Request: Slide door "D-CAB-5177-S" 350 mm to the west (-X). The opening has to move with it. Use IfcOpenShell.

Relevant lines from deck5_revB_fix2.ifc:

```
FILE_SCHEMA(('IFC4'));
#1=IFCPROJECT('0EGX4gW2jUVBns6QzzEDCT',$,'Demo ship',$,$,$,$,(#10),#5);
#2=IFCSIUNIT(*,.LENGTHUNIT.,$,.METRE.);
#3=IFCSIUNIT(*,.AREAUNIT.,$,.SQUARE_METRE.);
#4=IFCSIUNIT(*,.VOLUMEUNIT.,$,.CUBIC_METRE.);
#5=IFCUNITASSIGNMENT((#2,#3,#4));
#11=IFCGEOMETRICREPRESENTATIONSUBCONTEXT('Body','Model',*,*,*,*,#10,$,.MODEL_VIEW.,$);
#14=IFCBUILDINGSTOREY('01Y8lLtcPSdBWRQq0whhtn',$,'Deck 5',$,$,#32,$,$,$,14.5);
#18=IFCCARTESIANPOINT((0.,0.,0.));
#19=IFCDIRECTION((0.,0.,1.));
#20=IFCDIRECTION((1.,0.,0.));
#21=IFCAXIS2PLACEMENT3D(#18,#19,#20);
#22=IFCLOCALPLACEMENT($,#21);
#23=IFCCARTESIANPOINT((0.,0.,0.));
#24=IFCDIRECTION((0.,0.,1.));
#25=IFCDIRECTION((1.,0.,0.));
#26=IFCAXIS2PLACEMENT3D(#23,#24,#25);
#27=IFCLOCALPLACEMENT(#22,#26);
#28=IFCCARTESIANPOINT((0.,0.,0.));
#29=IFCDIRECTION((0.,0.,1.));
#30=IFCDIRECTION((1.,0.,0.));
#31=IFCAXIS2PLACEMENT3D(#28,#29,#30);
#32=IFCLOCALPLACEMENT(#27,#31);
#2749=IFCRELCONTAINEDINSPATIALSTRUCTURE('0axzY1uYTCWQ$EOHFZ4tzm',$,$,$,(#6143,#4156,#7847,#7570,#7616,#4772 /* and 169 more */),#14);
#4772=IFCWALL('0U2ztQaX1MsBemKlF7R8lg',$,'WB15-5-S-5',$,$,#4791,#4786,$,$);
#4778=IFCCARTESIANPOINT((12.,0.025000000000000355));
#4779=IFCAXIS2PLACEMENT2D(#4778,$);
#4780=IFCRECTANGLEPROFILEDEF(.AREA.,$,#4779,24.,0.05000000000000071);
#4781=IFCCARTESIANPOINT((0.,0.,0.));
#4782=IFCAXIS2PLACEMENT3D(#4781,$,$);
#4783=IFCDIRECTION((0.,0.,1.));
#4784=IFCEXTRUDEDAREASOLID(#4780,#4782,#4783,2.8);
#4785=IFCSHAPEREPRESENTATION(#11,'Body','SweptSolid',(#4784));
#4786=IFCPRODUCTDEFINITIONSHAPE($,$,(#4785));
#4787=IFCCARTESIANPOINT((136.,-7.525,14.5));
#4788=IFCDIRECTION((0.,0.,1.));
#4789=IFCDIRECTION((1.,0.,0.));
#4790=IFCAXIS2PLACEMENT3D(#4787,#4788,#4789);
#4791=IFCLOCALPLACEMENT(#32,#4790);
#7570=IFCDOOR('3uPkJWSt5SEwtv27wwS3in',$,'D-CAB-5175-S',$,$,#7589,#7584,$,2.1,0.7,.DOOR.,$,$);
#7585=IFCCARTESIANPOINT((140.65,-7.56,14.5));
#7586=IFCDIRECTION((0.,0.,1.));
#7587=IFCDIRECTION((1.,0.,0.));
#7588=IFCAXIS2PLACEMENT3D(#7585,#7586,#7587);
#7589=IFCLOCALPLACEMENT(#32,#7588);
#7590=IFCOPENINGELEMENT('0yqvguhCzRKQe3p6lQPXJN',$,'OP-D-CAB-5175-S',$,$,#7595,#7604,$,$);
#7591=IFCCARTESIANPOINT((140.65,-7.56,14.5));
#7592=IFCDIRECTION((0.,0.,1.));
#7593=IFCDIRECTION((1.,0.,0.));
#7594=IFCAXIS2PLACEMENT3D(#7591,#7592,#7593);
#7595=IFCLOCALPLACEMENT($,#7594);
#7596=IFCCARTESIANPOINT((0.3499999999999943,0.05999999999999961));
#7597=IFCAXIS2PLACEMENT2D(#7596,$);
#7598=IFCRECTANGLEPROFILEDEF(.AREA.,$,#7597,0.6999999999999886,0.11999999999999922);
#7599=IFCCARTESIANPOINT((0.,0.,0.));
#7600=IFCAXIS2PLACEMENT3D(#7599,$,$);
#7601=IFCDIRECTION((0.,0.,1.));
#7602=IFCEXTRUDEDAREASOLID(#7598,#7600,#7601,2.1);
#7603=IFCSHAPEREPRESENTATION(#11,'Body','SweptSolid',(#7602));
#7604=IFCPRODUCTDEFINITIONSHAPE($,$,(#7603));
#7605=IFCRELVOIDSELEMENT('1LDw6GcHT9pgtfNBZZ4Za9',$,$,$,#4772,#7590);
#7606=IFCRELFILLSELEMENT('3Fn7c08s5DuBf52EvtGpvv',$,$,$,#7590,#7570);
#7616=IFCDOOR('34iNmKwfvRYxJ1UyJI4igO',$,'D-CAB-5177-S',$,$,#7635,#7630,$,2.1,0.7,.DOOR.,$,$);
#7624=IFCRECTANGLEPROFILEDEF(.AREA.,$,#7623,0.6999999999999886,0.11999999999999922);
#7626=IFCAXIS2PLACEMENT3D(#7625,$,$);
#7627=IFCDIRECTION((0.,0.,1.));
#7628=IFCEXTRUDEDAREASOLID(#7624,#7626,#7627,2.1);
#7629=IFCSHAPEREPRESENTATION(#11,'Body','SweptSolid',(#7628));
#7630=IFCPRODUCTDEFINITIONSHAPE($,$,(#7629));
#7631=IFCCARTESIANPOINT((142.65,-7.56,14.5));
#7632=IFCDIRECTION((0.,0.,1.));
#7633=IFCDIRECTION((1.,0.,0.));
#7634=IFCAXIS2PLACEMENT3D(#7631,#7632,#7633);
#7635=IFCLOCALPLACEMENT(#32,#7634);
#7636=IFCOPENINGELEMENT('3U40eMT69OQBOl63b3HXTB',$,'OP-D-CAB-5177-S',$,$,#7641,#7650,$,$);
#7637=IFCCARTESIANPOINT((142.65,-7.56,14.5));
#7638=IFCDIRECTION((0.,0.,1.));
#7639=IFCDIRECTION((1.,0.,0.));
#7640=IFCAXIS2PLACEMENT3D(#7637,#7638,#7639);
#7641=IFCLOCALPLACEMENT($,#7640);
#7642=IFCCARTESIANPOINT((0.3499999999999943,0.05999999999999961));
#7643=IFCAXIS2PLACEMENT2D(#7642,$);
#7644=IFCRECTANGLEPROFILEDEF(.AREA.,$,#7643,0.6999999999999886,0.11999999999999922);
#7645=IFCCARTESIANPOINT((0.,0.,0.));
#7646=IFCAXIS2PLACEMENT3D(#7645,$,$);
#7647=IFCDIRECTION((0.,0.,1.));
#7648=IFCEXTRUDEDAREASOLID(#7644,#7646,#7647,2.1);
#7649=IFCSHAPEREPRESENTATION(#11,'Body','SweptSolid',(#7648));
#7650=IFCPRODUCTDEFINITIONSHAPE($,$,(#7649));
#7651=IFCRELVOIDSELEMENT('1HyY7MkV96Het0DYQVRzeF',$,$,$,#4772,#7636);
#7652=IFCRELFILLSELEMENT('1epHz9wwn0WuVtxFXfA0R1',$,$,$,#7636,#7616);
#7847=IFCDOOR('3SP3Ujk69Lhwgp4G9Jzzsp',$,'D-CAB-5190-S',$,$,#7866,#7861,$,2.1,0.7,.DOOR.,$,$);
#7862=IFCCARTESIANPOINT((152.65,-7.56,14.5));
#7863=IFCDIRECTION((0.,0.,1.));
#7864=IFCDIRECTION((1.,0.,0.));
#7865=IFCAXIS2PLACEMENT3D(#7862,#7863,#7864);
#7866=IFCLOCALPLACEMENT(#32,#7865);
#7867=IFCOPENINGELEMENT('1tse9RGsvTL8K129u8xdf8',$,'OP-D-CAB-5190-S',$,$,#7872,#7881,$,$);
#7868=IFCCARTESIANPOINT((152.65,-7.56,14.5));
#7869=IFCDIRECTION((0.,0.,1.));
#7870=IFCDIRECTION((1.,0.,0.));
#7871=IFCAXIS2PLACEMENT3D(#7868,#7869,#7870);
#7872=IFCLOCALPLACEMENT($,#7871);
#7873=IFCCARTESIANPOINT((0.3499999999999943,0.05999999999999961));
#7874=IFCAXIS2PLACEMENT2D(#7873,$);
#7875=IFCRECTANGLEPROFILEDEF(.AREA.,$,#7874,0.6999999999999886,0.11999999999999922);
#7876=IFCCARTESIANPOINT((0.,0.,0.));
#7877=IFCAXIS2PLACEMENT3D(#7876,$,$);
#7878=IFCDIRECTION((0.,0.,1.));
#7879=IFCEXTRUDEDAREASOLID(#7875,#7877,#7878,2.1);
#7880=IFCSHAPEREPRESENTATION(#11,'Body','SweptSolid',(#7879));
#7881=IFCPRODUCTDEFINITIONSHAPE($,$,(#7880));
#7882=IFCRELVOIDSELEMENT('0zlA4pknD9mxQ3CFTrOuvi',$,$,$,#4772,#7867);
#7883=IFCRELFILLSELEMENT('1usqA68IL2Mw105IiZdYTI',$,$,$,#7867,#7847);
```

```python
import ifcopenshell
import ifcopenshell.api.geometry
import ifcopenshell.util.placement

model = ifcopenshell.open("deck5_revB_fix2.ifc")

door = model.by_id(7616)
opening = door.FillsVoids[0].RelatingOpeningElement
wall = opening.VoidsElements[0].RelatingBuildingElement

wall_matrix = ifcopenshell.util.placement.get_local_placement(wall.ObjectPlacement)
shift = wall_matrix[:3, 0] * -0.35
before = ifcopenshell.util.placement.get_local_placement(door.ObjectPlacement)[:3, 3].copy()

# The door is not placed relative to its opening, so move both.
for product in (opening, door):
    matrix = ifcopenshell.util.placement.get_local_placement(product.ObjectPlacement)
    matrix[:3, 3] += shift
    ifcopenshell.api.geometry.edit_object_placement(model, product=product, matrix=matrix, is_si=False)

after = ifcopenshell.util.placement.get_local_placement(door.ObjectPlacement)[:3, 3]
print("door moved by", (after - before).round(3) + 0.0)

model.write("deck5_revB_fix2_v2.ifc")
```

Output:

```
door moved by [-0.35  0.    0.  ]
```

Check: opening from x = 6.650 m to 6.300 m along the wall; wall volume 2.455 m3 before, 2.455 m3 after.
